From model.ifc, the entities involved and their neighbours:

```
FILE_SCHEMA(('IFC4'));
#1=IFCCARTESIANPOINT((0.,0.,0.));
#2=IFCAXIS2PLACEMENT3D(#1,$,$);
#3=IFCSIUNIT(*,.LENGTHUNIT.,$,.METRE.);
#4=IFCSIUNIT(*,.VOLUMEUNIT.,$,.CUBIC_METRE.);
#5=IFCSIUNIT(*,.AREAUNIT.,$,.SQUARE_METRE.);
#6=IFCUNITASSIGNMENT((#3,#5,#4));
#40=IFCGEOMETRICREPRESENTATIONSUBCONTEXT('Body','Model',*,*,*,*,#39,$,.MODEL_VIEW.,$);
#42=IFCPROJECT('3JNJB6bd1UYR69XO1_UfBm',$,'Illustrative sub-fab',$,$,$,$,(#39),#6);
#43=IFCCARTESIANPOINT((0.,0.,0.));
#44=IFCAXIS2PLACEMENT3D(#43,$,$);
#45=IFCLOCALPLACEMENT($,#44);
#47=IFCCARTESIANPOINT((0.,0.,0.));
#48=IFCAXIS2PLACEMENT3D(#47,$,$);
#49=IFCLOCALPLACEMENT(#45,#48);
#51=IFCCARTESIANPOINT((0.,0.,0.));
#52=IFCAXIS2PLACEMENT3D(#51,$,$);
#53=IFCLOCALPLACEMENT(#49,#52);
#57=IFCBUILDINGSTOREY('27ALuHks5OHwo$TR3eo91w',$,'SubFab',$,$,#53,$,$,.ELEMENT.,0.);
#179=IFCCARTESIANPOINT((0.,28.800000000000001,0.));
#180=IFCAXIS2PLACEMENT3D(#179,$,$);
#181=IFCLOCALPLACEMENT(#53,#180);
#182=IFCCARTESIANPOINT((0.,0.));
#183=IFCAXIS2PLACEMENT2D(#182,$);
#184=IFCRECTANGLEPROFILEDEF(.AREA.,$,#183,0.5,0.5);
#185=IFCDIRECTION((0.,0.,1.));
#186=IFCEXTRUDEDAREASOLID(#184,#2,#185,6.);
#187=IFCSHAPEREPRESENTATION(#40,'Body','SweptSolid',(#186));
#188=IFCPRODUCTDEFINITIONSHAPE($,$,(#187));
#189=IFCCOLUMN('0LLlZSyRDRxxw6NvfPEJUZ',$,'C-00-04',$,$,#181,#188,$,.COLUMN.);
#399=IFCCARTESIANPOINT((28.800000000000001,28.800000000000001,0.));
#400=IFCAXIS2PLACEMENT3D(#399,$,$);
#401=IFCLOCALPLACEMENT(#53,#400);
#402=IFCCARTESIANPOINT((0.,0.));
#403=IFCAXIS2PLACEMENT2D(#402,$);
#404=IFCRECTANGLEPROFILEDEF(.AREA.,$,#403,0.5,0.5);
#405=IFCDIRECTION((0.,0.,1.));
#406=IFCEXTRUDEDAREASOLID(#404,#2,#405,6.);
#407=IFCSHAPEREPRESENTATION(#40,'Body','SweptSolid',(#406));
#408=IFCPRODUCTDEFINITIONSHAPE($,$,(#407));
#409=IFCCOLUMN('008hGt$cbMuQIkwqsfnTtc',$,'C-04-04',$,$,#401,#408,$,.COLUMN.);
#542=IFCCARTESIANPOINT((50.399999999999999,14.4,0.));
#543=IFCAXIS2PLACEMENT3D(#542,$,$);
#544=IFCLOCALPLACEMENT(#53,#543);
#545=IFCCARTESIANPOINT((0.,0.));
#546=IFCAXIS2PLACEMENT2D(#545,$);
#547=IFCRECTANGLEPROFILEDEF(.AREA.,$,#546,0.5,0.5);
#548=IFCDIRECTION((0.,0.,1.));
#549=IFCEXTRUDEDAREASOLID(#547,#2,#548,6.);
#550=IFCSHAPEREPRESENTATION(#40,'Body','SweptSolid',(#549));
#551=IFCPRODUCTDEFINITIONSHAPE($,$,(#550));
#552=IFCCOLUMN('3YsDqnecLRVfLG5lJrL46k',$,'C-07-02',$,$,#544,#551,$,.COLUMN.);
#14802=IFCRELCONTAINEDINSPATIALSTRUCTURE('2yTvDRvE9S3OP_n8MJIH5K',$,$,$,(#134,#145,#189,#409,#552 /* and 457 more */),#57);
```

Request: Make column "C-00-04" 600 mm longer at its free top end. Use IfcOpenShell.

```python
import ifcopenshell
import ifcopenshell.util.representation
import ifcopenshell.util.unit

model = ifcopenshell.open("model.ifc")
unit_scale = ifcopenshell.util.unit.calculate_unit_scale(model)

member = model.by_guid("0LLlZSyRDRxxw6NvfPEJUZ")
change = 0.6 / unit_scale

# The extrusion runs towards the end named, so only its depth changes.
body = ifcopenshell.util.representation.get_representation(member, "Model", "Body")
solid = body.Items[0]
old_length = solid.Depth
solid.Depth += change

print(f"length {old_length:g} -> {solid.Depth:g}")

model.write("model_v2.ifc")
```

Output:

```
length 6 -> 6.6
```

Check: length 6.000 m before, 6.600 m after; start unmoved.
